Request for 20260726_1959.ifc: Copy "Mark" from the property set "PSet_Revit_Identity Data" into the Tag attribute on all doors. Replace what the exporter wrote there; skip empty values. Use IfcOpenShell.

First a look at what the model holds.

```python
import ifcopenshell
import ifcopenshell.util.element

model = ifcopenshell.open("20260726_1959.ifc")
print(model.schema)
doors = model.by_type("IfcDoor")
print(len(doors), "doors")
for e in doors[:8]:
    source = ifcopenshell.util.element.get_pset(e, "PSet_Revit_Identity Data", "Mark")
    target = e.Tag
    print(e.id(), repr(source), repr(target), sep=" | ")
```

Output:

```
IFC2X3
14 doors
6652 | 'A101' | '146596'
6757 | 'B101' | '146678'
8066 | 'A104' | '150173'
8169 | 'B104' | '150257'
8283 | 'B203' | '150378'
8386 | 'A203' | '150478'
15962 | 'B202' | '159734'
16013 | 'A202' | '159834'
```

```python
import ifcopenshell
import ifcopenshell.util.element

model = ifcopenshell.open("20260726_1959.ifc")

count = 0
for e in model.by_type("IfcDoor"):
    value = ifcopenshell.util.element.get_pset(e, "PSet_Revit_Identity Data", "Mark")
    current = e.Tag
    if not value or not value.strip() or current == value:
        continue
    e.Tag = value
    count += 1

print(count, "doors updated")

model.write("20260726_1959_updated.ifc")
```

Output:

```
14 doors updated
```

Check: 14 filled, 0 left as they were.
